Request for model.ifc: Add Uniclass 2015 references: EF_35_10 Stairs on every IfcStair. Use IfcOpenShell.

First a look at what the model holds.

```python
import ifcopenshell

model = ifcopenshell.open("model.ifc")
print(model.schema)
print("classifications:", [c.Name for c in model.by_type("IfcClassification")])
for ifc_class in ("IfcDoor", "IfcRoof", "IfcStair", "IfcWall", "IfcWindow"):
    print(ifc_class, len(model.by_type(ifc_class)))
```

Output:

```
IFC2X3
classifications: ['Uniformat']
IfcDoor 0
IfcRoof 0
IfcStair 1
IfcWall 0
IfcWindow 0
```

```python
import ifcopenshell
import ifcopenshell.api.classification

model = ifcopenshell.open("model.ifc")

# IFC2X3 requires Source and Edition and has no link from the project to the system.
system = model.create_entity("IfcClassification", Source="NBS", Edition="2015", Name="Uniclass 2015")

codes = {
    "IfcStair": ("EF_35_10", "Stairs"),
}
for ifc_class, (code, name) in codes.items():
    products = model.by_type(ifc_class)
    ifcopenshell.api.classification.add_reference(
        model, products=products, classification=system, identification=code, name=name
    )
    print(code, len(products))

model.write("model_edited.ifc")
```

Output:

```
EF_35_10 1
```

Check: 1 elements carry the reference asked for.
